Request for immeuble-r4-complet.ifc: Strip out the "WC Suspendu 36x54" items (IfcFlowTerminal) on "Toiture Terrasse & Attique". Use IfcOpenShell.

First a look at what the model holds.

```python
import ifcopenshell
import ifcopenshell.util.element

model = ifcopenshell.open("immeuble-r4-complet.ifc")
print(model.schema)
storey = next(s for s in model.by_type("IfcBuildingStorey") if s.Name == "Toiture Terrasse & Attique")
terminals = [e for e in ifcopenshell.util.element.get_decomposition(storey) if e.is_a("IfcFlowTerminal")]
seen = {}
for e in terminals:
    element_type = ifcopenshell.util.element.get_type(e)
    name = element_type.Name if element_type not in (None, e) else None
    seen[name] = seen.get(name, 0) + 1
for name, count in sorted(seen.items(), key=str):
    print(count, "x", name)
```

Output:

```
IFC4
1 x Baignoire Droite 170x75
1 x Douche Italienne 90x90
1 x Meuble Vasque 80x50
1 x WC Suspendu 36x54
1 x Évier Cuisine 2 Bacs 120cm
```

```python
import ifcopenshell
import ifcopenshell.api.root
import ifcopenshell.util.element

model = ifcopenshell.open("immeuble-r4-complet.ifc")

storey = next(s for s in model.by_type("IfcBuildingStorey") if s.Name == "Toiture Terrasse & Attique")
terminals = [e for e in ifcopenshell.util.element.get_decomposition(storey) if e.is_a("IfcFlowTerminal")]
targets = [e for e in terminals if (t := ifcopenshell.util.element.get_type(e)) not in (None, e) and t.Name == "WC Suspendu 36x54"]

for e in targets:
    ifcopenshell.api.root.remove_product(model, product=e)
print(len(targets), "removed")

model.write("immeuble-r4-complet_rev.ifc")
```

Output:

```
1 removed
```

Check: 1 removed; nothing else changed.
